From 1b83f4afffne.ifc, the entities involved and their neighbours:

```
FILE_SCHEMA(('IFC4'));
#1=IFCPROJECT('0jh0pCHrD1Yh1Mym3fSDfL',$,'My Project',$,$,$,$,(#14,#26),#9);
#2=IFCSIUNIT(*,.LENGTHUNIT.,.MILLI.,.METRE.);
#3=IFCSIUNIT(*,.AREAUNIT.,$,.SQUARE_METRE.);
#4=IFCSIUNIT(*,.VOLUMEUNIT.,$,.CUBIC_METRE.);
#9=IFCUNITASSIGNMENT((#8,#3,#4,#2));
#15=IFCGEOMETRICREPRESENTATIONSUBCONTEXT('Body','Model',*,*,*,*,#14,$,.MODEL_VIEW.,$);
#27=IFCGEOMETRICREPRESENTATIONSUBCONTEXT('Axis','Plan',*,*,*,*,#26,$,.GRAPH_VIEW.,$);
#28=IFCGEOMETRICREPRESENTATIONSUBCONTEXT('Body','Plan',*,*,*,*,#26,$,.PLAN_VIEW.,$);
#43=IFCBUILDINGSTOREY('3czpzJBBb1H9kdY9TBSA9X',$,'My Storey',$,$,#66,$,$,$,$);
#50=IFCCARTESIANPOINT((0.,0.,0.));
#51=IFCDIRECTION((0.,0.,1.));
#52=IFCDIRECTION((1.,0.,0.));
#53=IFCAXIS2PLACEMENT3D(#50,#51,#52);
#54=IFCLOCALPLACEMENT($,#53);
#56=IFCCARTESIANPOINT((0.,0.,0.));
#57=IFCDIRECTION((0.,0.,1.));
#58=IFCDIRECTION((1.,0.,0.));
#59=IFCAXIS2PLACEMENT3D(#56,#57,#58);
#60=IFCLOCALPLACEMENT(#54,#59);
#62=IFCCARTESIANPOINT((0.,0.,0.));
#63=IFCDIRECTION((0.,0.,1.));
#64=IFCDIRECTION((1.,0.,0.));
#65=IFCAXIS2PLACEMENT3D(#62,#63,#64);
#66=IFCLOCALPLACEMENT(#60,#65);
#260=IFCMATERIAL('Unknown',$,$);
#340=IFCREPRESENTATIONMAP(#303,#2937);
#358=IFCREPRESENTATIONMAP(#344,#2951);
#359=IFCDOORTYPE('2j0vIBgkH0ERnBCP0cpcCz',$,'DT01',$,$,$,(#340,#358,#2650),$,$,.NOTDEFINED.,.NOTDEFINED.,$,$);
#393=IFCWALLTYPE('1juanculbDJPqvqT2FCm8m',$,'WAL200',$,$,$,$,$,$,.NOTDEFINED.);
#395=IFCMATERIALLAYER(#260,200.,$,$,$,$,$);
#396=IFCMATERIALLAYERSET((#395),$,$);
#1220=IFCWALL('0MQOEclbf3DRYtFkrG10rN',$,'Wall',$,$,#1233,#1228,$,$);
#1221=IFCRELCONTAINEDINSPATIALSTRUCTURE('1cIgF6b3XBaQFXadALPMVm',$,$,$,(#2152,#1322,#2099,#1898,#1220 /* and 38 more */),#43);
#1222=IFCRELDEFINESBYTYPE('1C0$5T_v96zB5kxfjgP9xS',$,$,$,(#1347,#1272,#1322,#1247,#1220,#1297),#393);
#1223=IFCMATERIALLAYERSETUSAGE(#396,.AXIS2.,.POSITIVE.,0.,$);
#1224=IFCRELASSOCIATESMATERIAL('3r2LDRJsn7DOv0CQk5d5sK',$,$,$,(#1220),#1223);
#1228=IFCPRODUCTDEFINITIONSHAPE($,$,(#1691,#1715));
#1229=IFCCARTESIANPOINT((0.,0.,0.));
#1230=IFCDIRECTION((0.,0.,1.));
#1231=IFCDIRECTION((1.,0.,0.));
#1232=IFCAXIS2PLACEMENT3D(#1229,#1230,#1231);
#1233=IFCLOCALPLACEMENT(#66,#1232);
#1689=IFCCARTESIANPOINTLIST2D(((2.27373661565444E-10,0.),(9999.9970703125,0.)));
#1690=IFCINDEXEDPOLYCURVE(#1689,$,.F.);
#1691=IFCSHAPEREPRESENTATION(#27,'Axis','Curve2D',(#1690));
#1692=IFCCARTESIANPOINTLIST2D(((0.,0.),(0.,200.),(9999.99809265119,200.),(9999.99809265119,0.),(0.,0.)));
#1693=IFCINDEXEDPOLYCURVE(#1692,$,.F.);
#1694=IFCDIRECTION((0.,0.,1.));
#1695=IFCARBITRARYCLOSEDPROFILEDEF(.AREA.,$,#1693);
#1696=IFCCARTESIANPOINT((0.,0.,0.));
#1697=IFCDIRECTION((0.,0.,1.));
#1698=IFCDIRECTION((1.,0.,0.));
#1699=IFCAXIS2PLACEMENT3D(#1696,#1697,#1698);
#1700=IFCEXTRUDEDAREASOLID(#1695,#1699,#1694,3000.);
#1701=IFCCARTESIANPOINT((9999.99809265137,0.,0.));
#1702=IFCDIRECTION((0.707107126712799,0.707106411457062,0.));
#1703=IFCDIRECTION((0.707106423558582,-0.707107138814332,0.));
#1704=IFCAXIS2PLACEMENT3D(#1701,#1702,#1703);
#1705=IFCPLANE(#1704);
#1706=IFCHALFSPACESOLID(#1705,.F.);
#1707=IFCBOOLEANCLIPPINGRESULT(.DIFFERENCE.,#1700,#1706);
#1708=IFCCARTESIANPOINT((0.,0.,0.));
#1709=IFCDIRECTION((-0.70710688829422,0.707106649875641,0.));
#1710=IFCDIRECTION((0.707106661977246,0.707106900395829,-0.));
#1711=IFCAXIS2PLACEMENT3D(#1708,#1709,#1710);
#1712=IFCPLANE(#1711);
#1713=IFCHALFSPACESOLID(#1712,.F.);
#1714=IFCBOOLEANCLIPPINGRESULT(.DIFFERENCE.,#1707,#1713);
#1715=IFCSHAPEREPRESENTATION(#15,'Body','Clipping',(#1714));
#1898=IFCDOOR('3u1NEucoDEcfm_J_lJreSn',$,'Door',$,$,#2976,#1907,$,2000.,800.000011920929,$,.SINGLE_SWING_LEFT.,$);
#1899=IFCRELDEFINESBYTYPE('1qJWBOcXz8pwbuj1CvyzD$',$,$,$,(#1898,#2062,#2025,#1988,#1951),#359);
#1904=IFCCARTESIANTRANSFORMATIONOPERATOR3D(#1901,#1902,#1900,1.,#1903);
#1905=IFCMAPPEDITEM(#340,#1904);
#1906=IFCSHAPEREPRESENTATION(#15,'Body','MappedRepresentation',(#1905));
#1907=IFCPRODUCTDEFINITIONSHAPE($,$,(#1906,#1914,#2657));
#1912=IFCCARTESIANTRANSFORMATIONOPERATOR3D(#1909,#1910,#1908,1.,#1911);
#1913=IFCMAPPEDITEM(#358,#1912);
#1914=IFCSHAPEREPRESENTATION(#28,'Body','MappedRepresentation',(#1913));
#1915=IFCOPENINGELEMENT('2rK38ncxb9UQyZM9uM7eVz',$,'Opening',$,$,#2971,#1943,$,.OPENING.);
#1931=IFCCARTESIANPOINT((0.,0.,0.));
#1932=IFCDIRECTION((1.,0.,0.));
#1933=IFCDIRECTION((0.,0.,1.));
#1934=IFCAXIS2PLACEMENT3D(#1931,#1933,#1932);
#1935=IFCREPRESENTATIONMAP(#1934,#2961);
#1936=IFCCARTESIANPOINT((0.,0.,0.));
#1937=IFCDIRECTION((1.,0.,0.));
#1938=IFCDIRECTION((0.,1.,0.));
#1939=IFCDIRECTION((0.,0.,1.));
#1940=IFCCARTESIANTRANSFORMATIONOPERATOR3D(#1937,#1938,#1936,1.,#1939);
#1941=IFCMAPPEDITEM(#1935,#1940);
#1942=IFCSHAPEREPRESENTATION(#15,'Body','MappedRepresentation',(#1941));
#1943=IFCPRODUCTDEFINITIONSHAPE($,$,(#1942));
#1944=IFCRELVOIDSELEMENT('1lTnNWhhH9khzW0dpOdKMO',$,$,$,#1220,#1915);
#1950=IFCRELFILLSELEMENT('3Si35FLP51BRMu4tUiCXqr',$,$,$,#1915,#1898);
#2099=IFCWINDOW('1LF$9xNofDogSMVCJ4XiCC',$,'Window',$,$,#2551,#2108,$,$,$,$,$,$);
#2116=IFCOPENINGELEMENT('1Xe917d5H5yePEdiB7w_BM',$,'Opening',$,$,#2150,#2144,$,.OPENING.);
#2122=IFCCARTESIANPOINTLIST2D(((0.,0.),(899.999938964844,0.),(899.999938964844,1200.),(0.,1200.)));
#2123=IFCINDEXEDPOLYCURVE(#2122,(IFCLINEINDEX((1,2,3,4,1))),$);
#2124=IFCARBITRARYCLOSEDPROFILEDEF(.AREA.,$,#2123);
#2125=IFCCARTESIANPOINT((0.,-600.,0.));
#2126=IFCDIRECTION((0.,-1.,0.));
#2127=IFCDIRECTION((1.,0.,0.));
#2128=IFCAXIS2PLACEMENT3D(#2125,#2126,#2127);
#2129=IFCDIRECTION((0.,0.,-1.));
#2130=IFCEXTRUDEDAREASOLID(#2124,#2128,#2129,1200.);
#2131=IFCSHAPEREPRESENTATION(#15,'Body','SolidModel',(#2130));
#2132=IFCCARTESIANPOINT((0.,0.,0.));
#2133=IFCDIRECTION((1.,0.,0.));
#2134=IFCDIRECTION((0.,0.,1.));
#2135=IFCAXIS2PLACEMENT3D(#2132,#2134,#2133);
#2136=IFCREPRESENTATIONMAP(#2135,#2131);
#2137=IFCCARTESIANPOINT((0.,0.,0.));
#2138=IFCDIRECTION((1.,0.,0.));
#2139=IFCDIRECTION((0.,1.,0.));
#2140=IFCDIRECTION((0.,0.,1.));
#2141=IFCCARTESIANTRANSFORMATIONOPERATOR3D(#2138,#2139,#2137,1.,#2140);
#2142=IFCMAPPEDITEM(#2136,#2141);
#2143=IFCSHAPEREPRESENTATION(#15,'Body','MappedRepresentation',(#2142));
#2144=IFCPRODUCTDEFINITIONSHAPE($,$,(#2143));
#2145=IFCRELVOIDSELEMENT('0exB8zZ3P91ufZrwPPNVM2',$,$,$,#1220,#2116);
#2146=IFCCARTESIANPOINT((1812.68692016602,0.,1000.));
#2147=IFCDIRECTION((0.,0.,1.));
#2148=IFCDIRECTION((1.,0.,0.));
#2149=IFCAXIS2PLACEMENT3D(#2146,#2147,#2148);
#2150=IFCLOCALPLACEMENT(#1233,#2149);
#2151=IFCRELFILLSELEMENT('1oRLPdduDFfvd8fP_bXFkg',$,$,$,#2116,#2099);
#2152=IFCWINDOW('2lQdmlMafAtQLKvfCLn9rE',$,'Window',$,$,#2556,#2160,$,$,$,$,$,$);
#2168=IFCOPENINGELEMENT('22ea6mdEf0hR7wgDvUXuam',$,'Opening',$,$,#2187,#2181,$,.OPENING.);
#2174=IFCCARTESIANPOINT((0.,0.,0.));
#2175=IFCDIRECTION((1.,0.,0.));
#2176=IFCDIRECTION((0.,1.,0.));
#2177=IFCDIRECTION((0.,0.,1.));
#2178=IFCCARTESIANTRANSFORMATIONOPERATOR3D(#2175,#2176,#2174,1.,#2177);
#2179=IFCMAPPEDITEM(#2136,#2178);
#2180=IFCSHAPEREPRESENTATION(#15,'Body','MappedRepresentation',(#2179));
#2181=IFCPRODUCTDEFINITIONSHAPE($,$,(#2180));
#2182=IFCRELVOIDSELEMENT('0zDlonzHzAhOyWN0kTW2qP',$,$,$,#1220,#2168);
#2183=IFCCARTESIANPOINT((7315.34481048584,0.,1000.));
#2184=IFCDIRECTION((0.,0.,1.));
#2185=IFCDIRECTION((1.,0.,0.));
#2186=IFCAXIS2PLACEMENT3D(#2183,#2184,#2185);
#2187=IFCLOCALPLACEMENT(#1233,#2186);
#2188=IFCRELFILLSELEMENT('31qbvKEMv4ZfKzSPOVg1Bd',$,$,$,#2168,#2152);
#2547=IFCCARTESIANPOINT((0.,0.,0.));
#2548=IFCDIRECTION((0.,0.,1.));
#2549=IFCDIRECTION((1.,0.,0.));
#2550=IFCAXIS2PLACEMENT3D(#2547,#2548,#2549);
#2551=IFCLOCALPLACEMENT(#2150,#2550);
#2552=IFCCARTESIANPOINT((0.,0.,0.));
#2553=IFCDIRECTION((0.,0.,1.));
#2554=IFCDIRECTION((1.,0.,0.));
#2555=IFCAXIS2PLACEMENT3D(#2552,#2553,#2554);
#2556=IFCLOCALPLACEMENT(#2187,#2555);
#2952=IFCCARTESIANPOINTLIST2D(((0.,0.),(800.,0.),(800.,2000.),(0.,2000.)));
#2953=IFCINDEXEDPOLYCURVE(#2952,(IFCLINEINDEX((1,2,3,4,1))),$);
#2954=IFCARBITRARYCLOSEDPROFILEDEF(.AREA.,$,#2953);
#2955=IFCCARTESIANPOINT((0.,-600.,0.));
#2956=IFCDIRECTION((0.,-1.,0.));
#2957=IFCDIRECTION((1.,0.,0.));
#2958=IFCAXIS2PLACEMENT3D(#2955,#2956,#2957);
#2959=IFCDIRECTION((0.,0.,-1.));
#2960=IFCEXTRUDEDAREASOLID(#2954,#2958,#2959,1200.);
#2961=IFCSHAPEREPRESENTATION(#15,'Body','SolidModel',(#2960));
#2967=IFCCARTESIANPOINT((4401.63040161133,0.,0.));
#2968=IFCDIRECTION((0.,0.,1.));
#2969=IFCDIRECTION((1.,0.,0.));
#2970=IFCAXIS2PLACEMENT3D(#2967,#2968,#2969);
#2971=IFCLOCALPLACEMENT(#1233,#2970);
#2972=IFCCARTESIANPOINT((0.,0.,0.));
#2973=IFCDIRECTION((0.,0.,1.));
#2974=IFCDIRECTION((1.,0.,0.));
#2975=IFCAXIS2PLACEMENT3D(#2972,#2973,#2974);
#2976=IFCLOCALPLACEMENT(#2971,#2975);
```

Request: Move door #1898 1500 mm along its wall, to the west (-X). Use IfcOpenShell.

```python
import ifcopenshell
import ifcopenshell.api.geometry
import ifcopenshell.util.placement
import ifcopenshell.util.unit

model = ifcopenshell.open("1b83f4afffne.ifc")
unit_scale = ifcopenshell.util.unit.calculate_unit_scale(model)

door = model.by_guid("3u1NEucoDEcfm_J_lJreSn")
opening = door.FillsVoids[0].RelatingOpeningElement
wall = opening.VoidsElements[0].RelatingBuildingElement

wall_matrix = ifcopenshell.util.placement.get_local_placement(wall.ObjectPlacement)
shift = wall_matrix[:3, 0] * -1.5 / unit_scale
before = ifcopenshell.util.placement.get_local_placement(door.ObjectPlacement)[:3, 3].copy()

# The door is placed relative to its opening, so it follows when the opening moves.
matrix = ifcopenshell.util.placement.get_local_placement(opening.ObjectPlacement)
matrix[:3, 3] += shift
ifcopenshell.api.geometry.edit_object_placement(
    model, product=opening, matrix=matrix, is_si=False, should_transform_children=True
)

after = ifcopenshell.util.placement.get_local_placement(door.ObjectPlacement)[:3, 3]
print("door moved by", (after - before).round(3) + 0.0)

model.write("1b83f4afffne_edited.ifc")
```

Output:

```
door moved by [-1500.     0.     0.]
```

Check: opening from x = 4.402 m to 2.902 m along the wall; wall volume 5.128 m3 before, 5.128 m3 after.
